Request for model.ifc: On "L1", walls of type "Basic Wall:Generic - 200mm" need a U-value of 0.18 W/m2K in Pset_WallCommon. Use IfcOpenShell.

First a look at what the model holds.

```python
import ifcopenshell
import ifcopenshell.util.element

model = ifcopenshell.open("model.ifc")
print(model.schema)
storey = next(s for s in model.by_type("IfcBuildingStorey") if s.Name == "L1")
walls = [e for e in ifcopenshell.util.element.get_decomposition(storey) if e.is_a("IfcWall")]
seen = {}
for e in walls:
    element_type = ifcopenshell.util.element.get_type(e)
    key = (element_type.Name if element_type != e and element_type else None, ifcopenshell.util.element.get_pset(e, "Pset_WallCommon", "ThermalTransmittance"))
    seen[key] = seen.get(key, 0) + 1
for (name, value), count in sorted(seen.items(), key=str):
    print(count, "x", name, "|", value)
```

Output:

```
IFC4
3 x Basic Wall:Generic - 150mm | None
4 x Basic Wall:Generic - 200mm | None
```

```python
import ifcopenshell
import ifcopenshell.api.pset
import ifcopenshell.util.element

model = ifcopenshell.open("model.ifc")

storey = next(s for s in model.by_type("IfcBuildingStorey") if s.Name == "L1")
walls = [e for e in ifcopenshell.util.element.get_decomposition(storey) if e.is_a("IfcWall")]

count = 0
for e in walls:
    element_type = ifcopenshell.util.element.get_type(e)
    if element_type in (None, e) or element_type.Name != "Basic Wall:Generic - 200mm":
        continue
    # add_pset returns the element's existing set when there is one.
    pset = ifcopenshell.api.pset.add_pset(model, product=e, name="Pset_WallCommon")
    ifcopenshell.api.pset.edit_pset(model, pset=pset, properties={"ThermalTransmittance": 0.18})
    count += 1

print(count, "walls updated")

model.write("model_updated.ifc")
```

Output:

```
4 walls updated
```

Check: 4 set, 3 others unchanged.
